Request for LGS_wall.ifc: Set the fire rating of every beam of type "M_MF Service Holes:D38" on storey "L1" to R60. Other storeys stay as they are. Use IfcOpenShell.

First a look at what the model holds.

```python
import ifcopenshell
import ifcopenshell.util.element

model = ifcopenshell.open("LGS_wall.ifc")
print(model.schema)
storey = next(s for s in model.by_type("IfcBuildingStorey") if s.Name == "L1")
beams = [e for e in ifcopenshell.util.element.get_decomposition(storey) if e.is_a("IfcBeam")]
seen = {}
for e in beams:
    element_type = ifcopenshell.util.element.get_type(e)
    key = (element_type.Name if element_type != e and element_type else None, ifcopenshell.util.element.get_pset(e, "Pset_BeamCommon", "FireRating"))
    seen[key] = seen.get(key, 0) + 1
for (name, value), count in sorted(seen.items(), key=str):
    print(count, "x", name, "|", value)
```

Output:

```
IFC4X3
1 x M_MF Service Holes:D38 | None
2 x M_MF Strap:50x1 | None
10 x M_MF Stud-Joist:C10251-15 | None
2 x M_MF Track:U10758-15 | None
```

```python
import ifcopenshell
import ifcopenshell.api.pset
import ifcopenshell.util.element

model = ifcopenshell.open("LGS_wall.ifc")

storey = next(s for s in model.by_type("IfcBuildingStorey") if s.Name == "L1")
beams = [e for e in ifcopenshell.util.element.get_decomposition(storey) if e.is_a("IfcBeam")]

count = 0
for e in beams:
    element_type = ifcopenshell.util.element.get_type(e)
    if element_type in (None, e) or element_type.Name != "M_MF Service Holes:D38":
        continue
    # add_pset returns the element's existing set when there is one.
    pset = ifcopenshell.api.pset.add_pset(model, product=e, name="Pset_BeamCommon")
    ifcopenshell.api.pset.edit_pset(model, pset=pset, properties={"FireRating": "R60"})
    count += 1

print(count, "beams updated")

model.write("LGS_wall_updated.ifc")
```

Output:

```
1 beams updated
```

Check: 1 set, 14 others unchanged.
